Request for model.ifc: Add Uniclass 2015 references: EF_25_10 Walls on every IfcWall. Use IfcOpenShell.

First a look at what the model holds.

```python
import ifcopenshell

model = ifcopenshell.open("model.ifc")
print(model.schema)
print("classifications:", [c.Name for c in model.by_type("IfcClassification")])
for ifc_class in ("IfcDoor", "IfcRoof", "IfcStair", "IfcWall", "IfcWindow"):
    print(ifc_class, len(model.by_type(ifc_class)))
```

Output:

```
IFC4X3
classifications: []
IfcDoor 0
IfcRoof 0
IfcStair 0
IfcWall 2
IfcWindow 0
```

```python
import ifcopenshell
import ifcopenshell.api.classification

model = ifcopenshell.open("model.ifc")

system = ifcopenshell.api.classification.add_classification(model, classification="Uniclass 2015")

codes = {
    "IfcWall": ("EF_25_10", "Walls"),
}
for ifc_class, (code, name) in codes.items():
    products = model.by_type(ifc_class)
    ifcopenshell.api.classification.add_reference(
        model, products=products, classification=system, identification=code, name=name
    )
    print(code, len(products))

model.write("model_rev.ifc")
```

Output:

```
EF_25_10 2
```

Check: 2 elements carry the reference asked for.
